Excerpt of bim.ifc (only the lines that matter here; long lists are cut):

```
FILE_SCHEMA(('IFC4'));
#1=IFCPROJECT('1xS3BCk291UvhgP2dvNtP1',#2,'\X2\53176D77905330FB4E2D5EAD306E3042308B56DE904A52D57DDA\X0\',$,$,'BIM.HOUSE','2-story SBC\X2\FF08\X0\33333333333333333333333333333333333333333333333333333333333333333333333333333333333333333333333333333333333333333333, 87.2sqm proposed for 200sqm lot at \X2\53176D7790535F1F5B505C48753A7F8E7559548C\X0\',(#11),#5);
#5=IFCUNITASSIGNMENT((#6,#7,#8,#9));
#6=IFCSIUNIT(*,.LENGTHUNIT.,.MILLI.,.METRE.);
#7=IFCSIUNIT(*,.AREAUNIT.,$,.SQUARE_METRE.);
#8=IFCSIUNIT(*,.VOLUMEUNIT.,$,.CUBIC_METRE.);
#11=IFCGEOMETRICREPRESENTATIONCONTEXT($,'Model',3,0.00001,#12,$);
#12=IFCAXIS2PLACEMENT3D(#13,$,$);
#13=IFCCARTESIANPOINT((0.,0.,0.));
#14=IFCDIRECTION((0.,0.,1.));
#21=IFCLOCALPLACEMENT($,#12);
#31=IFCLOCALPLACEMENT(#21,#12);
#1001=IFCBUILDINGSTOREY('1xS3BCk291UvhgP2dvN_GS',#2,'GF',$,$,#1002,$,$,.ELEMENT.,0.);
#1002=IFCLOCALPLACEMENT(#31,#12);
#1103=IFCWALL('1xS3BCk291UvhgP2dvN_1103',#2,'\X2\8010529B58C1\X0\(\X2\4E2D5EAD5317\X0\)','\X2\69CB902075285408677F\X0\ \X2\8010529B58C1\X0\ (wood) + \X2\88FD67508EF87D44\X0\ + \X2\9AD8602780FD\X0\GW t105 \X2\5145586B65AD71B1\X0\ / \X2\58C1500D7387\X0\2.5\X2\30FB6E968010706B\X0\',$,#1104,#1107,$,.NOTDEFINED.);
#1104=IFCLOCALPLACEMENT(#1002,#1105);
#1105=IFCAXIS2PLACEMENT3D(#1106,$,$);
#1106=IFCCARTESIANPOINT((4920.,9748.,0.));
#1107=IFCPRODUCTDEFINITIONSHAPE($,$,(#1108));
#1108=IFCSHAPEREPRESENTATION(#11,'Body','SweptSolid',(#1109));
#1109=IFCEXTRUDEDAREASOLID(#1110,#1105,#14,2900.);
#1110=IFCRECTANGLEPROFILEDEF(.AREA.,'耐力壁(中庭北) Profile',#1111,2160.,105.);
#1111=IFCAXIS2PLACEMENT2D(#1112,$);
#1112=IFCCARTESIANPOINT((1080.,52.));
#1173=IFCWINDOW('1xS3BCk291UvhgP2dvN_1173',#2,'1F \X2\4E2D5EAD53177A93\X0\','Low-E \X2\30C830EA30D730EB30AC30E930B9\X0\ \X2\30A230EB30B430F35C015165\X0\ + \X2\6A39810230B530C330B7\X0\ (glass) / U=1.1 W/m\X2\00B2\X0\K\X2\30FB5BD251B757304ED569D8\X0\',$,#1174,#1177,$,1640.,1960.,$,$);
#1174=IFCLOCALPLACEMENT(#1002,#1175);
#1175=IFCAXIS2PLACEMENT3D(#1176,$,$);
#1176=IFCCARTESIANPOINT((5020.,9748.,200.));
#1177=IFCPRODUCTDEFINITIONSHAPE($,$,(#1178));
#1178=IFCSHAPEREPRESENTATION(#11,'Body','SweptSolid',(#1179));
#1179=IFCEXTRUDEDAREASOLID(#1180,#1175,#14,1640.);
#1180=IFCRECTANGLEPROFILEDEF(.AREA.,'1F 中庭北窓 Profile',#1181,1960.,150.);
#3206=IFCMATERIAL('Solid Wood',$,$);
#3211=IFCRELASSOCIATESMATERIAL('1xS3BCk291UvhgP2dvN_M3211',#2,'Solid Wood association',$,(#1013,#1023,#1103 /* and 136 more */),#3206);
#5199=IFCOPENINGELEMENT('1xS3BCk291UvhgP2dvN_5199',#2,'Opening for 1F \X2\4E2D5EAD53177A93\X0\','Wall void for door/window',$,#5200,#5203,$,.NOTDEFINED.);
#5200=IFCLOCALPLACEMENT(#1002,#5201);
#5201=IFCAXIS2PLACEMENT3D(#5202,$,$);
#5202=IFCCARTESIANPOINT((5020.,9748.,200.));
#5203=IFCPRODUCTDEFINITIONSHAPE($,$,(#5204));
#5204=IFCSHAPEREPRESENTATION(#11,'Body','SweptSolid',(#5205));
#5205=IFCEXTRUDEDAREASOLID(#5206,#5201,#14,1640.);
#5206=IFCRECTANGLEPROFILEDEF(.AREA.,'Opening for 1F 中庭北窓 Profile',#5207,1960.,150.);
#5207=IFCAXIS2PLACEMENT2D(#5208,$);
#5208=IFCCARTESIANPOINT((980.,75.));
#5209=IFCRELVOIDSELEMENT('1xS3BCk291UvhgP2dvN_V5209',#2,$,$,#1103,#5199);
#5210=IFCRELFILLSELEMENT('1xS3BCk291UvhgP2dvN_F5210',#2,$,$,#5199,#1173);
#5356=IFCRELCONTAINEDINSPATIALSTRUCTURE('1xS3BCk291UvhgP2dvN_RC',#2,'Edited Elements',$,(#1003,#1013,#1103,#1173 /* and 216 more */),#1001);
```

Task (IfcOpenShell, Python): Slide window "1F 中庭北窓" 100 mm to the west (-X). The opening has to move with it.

```python
import ifcopenshell
import ifcopenshell.api.geometry
import ifcopenshell.util.placement
import ifcopenshell.util.unit

model = ifcopenshell.open("bim.ifc")
unit_scale = ifcopenshell.util.unit.calculate_unit_scale(model)

window = model.by_guid("1xS3BCk291UvhgP2dvN_1173")
opening = window.FillsVoids[0].RelatingOpeningElement
wall = opening.VoidsElements[0].RelatingBuildingElement

wall_matrix = ifcopenshell.util.placement.get_local_placement(wall.ObjectPlacement)
shift = wall_matrix[:3, 0] * -0.1 / unit_scale
before = ifcopenshell.util.placement.get_local_placement(window.ObjectPlacement)[:3, 3].copy()

# The window is not placed relative to its opening, so move both.
for product in (opening, window):
    matrix = ifcopenshell.util.placement.get_local_placement(product.ObjectPlacement)
    matrix[:3, 3] += shift
    ifcopenshell.api.geometry.edit_object_placement(model, product=product, matrix=matrix, is_si=False)

after = ifcopenshell.util.placement.get_local_placement(window.ObjectPlacement)[:3, 3]
print("window moved by", (after - before).round(3) + 0.0)

model.write("bim_updated.ifc")
```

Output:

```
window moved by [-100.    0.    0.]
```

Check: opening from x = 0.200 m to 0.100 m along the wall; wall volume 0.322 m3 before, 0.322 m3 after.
